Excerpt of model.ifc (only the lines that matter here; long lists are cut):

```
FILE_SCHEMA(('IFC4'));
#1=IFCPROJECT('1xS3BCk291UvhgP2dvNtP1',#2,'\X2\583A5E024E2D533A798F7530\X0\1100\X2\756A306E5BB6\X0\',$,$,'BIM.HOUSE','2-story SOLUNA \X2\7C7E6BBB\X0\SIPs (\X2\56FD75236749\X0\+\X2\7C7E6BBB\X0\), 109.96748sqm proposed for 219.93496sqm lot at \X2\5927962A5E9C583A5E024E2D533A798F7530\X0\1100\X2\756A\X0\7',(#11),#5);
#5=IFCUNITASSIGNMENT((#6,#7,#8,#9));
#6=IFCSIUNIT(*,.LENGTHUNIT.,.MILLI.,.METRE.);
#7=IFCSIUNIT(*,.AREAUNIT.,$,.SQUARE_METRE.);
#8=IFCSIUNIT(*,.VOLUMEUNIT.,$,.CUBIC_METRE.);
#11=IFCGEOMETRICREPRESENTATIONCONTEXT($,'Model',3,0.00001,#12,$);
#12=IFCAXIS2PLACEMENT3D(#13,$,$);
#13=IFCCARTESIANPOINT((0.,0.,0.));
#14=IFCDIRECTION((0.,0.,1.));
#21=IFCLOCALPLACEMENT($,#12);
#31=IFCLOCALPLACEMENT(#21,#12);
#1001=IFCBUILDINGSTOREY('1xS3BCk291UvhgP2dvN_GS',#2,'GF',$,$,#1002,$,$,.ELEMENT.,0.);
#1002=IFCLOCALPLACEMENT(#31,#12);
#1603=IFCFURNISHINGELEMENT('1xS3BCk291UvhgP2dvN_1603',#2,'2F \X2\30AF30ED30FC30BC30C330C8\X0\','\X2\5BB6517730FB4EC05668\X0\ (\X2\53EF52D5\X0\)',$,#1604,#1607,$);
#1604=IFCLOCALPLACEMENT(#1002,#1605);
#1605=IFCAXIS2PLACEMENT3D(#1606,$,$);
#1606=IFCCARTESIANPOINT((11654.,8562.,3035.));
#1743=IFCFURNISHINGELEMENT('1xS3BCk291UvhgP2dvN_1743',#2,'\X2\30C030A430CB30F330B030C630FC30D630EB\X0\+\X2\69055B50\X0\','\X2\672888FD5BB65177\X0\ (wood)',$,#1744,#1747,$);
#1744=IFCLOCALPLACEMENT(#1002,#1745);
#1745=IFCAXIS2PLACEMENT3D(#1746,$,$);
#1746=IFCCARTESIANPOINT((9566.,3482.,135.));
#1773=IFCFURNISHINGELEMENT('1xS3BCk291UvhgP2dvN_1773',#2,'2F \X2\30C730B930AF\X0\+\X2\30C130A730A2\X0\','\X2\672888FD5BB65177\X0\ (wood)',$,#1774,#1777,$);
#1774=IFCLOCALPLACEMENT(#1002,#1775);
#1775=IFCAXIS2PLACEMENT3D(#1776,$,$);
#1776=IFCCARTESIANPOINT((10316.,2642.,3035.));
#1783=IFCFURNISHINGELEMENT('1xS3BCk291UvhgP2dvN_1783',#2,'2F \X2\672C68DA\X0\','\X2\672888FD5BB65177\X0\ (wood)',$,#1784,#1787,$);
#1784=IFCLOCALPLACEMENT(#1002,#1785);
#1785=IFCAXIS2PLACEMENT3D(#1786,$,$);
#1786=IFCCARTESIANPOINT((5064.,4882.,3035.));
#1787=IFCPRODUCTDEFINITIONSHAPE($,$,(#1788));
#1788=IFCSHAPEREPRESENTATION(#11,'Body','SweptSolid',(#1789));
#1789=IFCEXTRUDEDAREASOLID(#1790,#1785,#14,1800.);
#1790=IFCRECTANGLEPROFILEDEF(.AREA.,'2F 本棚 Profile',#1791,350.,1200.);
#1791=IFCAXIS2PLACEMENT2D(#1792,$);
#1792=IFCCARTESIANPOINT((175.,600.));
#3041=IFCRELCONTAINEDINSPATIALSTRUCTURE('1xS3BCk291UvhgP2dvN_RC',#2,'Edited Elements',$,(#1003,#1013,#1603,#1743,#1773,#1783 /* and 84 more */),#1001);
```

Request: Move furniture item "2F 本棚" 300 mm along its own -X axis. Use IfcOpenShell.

```python
import ifcopenshell
import ifcopenshell.api.geometry
import ifcopenshell.util.placement

model = ifcopenshell.open("model.ifc")

item = model.by_id(1783)
matrix = ifcopenshell.util.placement.get_local_placement(item.ObjectPlacement)
matrix[:3, 3] -= matrix[:3, 0] * 300.0
ifcopenshell.api.geometry.edit_object_placement(model, product=item, matrix=matrix, is_si=False)

print(ifcopenshell.util.placement.get_local_placement(item.ObjectPlacement).round(3) + 0.0)

model.write("model_rev.ifc")
```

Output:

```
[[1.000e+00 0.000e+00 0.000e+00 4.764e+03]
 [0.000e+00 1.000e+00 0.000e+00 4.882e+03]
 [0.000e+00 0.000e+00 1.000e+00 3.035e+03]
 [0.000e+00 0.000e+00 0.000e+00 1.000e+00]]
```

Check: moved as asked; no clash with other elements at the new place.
